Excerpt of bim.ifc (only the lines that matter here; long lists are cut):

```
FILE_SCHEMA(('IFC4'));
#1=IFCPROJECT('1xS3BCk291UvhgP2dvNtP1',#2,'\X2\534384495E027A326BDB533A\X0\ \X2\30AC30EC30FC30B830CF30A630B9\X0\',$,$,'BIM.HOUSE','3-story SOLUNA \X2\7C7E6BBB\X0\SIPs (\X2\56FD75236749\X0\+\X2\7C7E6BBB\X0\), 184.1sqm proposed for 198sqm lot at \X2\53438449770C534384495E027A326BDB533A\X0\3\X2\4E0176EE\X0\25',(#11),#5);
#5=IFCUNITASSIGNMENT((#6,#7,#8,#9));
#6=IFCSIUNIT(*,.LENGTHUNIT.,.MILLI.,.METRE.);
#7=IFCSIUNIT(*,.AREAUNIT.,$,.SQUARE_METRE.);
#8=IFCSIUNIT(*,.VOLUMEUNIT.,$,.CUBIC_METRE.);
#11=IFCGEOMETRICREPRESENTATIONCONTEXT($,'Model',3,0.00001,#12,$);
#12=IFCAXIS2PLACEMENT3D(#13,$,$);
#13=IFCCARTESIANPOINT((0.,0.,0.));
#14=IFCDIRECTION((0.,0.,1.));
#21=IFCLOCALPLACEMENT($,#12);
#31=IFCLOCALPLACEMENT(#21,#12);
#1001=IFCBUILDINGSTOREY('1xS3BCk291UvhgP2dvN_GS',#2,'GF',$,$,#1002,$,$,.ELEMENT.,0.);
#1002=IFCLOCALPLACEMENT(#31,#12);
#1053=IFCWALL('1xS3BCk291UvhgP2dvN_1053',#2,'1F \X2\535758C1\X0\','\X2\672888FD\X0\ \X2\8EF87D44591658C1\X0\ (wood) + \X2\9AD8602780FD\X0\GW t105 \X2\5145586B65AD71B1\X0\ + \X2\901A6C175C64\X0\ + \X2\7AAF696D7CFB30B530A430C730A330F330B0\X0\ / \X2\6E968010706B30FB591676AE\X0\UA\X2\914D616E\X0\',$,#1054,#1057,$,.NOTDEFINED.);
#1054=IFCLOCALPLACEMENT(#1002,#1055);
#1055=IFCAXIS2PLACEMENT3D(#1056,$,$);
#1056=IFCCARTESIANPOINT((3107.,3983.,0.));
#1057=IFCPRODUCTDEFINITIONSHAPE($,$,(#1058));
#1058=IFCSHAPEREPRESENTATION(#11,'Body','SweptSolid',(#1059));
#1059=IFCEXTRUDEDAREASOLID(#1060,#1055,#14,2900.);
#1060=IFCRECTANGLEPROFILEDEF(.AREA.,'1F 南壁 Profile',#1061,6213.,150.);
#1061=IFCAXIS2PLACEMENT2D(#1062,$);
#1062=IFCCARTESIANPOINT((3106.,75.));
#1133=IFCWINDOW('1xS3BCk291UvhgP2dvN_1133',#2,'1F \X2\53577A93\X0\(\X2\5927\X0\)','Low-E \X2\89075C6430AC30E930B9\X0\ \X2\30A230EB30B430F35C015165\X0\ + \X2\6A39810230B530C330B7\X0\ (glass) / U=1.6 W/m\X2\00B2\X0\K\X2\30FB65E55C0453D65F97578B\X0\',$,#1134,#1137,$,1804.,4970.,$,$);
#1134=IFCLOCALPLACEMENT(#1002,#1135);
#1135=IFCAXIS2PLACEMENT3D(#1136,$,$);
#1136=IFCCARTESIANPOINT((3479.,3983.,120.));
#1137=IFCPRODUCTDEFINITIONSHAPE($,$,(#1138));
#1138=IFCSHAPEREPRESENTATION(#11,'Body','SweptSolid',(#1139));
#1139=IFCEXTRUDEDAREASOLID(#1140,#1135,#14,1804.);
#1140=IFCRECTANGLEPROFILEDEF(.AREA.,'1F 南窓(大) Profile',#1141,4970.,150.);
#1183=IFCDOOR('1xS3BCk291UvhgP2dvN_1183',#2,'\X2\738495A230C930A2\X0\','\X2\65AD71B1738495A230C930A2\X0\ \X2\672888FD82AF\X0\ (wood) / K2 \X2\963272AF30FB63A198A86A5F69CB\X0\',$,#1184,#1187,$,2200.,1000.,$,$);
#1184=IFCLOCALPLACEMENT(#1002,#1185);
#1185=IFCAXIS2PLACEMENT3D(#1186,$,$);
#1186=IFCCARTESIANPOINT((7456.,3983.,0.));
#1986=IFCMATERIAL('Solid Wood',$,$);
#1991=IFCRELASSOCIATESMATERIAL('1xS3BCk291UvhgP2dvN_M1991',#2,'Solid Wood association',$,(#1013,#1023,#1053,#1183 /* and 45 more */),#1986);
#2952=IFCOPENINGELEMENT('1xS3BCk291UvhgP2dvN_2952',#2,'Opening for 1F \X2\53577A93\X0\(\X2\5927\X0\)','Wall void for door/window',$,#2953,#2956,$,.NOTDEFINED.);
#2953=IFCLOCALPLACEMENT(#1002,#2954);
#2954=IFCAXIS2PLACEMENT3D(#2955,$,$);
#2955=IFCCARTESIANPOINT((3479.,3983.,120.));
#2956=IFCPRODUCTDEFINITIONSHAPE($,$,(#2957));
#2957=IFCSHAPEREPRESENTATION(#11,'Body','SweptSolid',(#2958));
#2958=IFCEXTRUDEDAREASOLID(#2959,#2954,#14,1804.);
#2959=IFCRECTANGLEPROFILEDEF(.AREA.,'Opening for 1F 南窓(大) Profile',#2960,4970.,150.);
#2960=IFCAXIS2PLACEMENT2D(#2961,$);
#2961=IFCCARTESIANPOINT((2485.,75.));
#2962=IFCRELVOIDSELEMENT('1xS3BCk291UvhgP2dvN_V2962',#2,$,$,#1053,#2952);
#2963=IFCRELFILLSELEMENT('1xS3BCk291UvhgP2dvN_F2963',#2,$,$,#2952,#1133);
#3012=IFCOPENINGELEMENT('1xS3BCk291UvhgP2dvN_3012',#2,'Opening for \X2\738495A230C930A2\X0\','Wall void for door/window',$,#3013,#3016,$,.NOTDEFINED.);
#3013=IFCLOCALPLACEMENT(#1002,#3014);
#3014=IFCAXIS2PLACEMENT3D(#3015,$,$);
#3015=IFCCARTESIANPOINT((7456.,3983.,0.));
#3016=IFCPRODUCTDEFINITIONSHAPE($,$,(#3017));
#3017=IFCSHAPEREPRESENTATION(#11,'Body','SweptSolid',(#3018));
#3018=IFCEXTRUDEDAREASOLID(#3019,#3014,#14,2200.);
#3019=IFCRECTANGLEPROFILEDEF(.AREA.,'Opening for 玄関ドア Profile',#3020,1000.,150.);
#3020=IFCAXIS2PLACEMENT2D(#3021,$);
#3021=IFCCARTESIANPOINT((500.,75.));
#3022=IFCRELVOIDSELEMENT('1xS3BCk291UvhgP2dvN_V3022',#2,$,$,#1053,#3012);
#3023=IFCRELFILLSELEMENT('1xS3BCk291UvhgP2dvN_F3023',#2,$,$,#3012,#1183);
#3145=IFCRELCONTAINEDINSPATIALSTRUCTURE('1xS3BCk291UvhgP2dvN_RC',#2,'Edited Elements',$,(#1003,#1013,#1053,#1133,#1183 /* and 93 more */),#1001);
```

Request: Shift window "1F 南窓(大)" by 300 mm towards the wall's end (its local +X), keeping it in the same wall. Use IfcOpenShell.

```python
import ifcopenshell
import ifcopenshell.api.geometry
import ifcopenshell.util.placement
import ifcopenshell.util.unit

model = ifcopenshell.open("bim.ifc")
unit_scale = ifcopenshell.util.unit.calculate_unit_scale(model)

window = model.by_guid("1xS3BCk291UvhgP2dvN_1133")
opening = window.FillsVoids[0].RelatingOpeningElement
wall = opening.VoidsElements[0].RelatingBuildingElement

wall_matrix = ifcopenshell.util.placement.get_local_placement(wall.ObjectPlacement)
shift = wall_matrix[:3, 0] * 0.3 / unit_scale
before = ifcopenshell.util.placement.get_local_placement(window.ObjectPlacement)[:3, 3].copy()

# The window is not placed relative to its opening, so move both.
for product in (opening, window):
    matrix = ifcopenshell.util.placement.get_local_placement(product.ObjectPlacement)
    matrix[:3, 3] += shift
    ifcopenshell.api.geometry.edit_object_placement(model, product=product, matrix=matrix, is_si=False)

after = ifcopenshell.util.placement.get_local_placement(window.ObjectPlacement)[:3, 3]
print("window moved by", (after - before).round(3) + 0.0)

model.write("bim-out.ifc")
```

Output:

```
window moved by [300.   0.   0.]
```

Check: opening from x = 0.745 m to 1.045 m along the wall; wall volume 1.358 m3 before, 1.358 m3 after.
